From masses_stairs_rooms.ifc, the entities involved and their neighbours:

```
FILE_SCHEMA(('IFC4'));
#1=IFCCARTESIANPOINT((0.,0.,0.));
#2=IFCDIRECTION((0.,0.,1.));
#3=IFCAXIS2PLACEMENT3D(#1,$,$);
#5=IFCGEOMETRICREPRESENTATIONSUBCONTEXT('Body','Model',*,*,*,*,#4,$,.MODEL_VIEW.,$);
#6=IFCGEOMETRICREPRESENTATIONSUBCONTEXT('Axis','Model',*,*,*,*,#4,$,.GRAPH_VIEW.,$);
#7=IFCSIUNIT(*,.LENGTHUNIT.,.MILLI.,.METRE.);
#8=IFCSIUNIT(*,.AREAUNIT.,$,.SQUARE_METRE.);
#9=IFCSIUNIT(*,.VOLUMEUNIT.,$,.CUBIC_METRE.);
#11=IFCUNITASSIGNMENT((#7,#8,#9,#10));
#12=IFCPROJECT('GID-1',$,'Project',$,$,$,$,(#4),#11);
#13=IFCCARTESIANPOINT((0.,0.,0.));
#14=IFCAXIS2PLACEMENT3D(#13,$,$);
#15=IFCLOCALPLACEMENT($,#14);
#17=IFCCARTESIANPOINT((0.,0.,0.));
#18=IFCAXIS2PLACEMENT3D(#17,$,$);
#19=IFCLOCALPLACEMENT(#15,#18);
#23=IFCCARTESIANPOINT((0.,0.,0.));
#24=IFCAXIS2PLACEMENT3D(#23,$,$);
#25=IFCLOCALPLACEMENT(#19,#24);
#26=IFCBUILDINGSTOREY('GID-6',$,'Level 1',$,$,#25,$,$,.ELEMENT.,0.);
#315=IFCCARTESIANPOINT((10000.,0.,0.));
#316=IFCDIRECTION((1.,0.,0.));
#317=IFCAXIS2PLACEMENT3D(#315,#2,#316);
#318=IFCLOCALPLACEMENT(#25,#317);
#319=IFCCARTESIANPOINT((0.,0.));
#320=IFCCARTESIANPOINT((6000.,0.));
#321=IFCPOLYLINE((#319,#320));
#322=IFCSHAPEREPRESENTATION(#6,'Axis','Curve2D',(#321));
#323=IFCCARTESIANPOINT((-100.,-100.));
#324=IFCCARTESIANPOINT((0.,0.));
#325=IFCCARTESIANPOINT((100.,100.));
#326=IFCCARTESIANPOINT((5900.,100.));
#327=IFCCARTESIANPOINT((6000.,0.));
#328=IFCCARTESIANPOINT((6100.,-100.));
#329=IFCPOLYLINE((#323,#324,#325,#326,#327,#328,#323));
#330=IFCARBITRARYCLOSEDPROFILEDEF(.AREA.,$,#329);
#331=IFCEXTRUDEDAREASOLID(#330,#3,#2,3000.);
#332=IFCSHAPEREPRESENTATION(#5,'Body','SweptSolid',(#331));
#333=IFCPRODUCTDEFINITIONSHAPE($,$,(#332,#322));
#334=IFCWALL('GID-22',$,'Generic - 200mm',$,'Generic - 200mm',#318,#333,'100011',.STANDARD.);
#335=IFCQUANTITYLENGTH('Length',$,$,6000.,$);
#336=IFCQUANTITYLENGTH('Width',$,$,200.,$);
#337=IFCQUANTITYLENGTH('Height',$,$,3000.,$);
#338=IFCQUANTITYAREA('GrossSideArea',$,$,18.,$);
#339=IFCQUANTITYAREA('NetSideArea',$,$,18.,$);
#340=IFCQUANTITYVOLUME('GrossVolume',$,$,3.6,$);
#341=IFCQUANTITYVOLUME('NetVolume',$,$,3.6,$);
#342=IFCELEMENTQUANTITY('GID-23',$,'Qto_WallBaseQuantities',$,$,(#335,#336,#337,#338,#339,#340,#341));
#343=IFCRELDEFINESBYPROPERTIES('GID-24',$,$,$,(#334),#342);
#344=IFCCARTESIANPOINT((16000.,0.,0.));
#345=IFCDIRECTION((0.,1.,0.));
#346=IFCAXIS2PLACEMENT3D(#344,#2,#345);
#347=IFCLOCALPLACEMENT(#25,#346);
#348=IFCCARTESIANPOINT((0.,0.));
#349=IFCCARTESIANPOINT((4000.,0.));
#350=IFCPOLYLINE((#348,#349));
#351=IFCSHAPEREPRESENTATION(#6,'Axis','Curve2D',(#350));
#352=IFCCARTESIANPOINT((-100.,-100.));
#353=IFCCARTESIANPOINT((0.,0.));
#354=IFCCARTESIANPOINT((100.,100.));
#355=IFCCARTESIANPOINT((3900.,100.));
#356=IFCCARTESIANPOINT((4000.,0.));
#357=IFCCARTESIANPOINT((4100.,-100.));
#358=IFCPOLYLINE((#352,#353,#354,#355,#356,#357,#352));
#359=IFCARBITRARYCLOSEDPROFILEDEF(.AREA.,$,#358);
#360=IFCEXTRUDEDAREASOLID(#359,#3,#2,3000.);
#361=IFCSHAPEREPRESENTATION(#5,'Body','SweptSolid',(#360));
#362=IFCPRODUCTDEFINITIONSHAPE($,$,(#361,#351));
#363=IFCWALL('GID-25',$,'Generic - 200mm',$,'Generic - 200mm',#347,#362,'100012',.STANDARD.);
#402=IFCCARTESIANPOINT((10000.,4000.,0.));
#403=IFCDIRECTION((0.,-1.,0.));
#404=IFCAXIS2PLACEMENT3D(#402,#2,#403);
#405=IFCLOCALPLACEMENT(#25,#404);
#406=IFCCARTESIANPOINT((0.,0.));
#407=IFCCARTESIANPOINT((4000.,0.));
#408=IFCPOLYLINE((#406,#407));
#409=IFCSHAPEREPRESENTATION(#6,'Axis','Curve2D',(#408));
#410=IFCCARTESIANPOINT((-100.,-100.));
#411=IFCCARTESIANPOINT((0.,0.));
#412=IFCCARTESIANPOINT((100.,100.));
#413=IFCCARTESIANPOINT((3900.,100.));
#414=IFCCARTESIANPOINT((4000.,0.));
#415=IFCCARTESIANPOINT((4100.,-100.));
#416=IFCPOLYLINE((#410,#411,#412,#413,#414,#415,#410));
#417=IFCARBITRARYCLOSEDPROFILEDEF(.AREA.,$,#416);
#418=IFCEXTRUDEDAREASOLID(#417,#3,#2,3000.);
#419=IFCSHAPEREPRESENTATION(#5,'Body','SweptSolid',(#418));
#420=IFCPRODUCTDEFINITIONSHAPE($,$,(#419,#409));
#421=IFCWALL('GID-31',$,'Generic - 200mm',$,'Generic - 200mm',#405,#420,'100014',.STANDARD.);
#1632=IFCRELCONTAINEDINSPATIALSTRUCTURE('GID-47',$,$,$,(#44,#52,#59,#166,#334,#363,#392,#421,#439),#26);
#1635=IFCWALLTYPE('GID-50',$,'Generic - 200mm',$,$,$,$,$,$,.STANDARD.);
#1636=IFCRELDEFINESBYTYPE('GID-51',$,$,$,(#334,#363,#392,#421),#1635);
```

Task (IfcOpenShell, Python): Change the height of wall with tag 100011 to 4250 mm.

```python
import ifcopenshell
import ifcopenshell.api.pset
import ifcopenshell.geom
import ifcopenshell.util.element
import ifcopenshell.util.representation
import ifcopenshell.util.shape
import ifcopenshell.util.unit

model = ifcopenshell.open("masses_stairs_rooms.ifc")
unit_scale = ifcopenshell.util.unit.calculate_unit_scale(model)
area_scale = ifcopenshell.util.unit.calculate_unit_scale(model, "AREAUNIT")
volume_scale = ifcopenshell.util.unit.calculate_unit_scale(model, "VOLUMEUNIT")
settings = ifcopenshell.geom.settings()


def volume(element):
    """Net volume in cubic metres, openings subtracted."""
    shape = ifcopenshell.geom.create_shape(settings, element)
    return ifcopenshell.util.shape.get_volume(shape.geometry)


wall = model.by_id(334)
before = volume(wall)

body = ifcopenshell.util.representation.get_representation(wall, "Model", "Body")
solid = body.Items[0]
old_height = solid.Depth
solid.Depth = 4250.0
after = volume(wall)
thickness = 0.2  # wall thickness in metres

# Update the stored height, areas and volumes.
qto = model.by_id(ifcopenshell.util.element.get_pset(wall, "Qto_WallBaseQuantities", should_inherit=False)["id"])
ifcopenshell.api.pset.edit_qto(model, qto=qto, properties={
    "Height": solid.Depth,
    "GrossSideArea": ifcopenshell.util.element.get_pset(wall, "Qto_WallBaseQuantities", "GrossSideArea") * solid.Depth / old_height,
    "NetSideArea": after / thickness / area_scale,
    "GrossVolume": ifcopenshell.util.element.get_pset(wall, "Qto_WallBaseQuantities", "GrossVolume") * solid.Depth / old_height,
    "NetVolume": after / volume_scale,
})

print(f"height {old_height:g} -> {solid.Depth:g}, volume {before:.3f} -> {after:.3f} m3")

model.write("masses_stairs_rooms_updated.ifc")
```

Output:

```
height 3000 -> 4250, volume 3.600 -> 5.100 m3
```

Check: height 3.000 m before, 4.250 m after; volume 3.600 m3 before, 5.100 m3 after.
